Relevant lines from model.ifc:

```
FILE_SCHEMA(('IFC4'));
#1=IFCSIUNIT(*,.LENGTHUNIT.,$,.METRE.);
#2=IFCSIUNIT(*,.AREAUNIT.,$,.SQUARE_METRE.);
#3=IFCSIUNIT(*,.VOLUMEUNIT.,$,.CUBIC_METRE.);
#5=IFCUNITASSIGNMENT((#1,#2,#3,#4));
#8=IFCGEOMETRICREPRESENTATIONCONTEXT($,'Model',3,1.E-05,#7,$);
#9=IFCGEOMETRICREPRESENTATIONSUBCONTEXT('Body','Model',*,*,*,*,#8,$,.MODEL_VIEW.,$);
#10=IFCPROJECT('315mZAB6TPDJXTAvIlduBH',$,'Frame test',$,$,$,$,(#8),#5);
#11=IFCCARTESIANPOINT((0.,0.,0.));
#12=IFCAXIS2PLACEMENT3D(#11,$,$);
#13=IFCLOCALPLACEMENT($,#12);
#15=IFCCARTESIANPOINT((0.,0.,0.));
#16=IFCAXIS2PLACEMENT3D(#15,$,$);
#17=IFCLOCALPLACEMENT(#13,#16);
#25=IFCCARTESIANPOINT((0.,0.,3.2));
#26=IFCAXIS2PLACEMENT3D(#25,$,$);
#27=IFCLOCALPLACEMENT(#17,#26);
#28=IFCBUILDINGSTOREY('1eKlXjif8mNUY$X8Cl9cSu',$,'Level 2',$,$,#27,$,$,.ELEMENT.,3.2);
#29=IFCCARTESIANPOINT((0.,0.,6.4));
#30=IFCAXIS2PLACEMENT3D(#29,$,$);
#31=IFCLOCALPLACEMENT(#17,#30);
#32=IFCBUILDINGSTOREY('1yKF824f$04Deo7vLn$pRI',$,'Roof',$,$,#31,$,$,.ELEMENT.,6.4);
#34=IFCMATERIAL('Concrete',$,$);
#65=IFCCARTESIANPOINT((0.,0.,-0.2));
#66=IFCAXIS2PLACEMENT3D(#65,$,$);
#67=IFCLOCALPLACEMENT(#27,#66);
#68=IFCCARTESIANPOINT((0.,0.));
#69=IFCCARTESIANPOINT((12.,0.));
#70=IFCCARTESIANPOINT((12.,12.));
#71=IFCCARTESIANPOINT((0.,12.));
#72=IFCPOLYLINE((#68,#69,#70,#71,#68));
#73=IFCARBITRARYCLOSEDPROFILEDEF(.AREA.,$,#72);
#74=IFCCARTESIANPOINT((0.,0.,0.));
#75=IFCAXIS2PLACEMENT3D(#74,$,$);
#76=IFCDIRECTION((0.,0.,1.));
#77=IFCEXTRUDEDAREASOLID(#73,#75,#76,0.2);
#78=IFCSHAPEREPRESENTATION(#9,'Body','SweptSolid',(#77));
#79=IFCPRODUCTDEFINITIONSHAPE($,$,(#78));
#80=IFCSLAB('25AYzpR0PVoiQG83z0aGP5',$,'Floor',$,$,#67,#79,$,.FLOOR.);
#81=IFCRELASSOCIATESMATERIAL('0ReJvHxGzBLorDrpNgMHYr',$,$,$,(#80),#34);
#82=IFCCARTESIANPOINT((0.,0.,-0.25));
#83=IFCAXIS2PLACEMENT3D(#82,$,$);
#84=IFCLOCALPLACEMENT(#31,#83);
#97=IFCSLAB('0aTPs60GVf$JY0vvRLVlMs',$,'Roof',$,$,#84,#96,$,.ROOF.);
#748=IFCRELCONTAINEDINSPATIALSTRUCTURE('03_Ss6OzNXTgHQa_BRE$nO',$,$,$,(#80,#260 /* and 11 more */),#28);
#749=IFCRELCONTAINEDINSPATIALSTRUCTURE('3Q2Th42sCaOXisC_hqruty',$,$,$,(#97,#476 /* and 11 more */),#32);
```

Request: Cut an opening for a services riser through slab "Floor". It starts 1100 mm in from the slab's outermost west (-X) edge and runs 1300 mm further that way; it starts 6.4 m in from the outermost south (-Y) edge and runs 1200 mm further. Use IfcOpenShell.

```python
import numpy as np
import ifcopenshell
import ifcopenshell.api.feature
import ifcopenshell.api.geometry
import ifcopenshell.api.root
import ifcopenshell.geom
import ifcopenshell.util.placement
import ifcopenshell.util.representation
import ifcopenshell.util.shape
import ifcopenshell.util.unit

model = ifcopenshell.open("model.ifc")
unit_scale = ifcopenshell.util.unit.calculate_unit_scale(model)
settings = ifcopenshell.geom.settings()


def volume(element):
    """Net volume in cubic metres, openings subtracted."""
    shape = ifcopenshell.geom.create_shape(settings, element)
    return ifcopenshell.util.shape.get_volume(shape.geometry)


slab = model.by_guid("25AYzpR0PVoiQG83z0aGP5")
before = volume(slab)

# Extent in the slab's own axes, in metres. The edges named are its -X and -Y sides.
slab_shape = ifcopenshell.geom.create_shape(settings, slab)
vertices = ifcopenshell.util.shape.get_vertices(slab_shape.geometry)
x_min, y_min, bottom = vertices.min(axis=0)
top = vertices[:, 2].max()

opening = ifcopenshell.api.root.create_entity(model, ifc_class="IfcOpeningElement", name="Services riser opening", predefined_type="OPENING")
context = ifcopenshell.util.representation.get_context(model, "Model", "Body", "MODEL_VIEW")
width, depth = 1.3, 1.2
outline = [(0.0, 0.0), (width, 0.0), (width, depth), (0.0, depth), (0.0, 0.0)]
# Overshoot both faces by 50 mm so the cut is clean.
shape = ifcopenshell.api.geometry.add_slab_representation(
    model, context=context, depth=top - bottom + 0.1, polyline=outline
)
ifcopenshell.api.geometry.assign_representation(model, product=opening, representation=shape)

matrix = ifcopenshell.util.placement.get_local_placement(slab.ObjectPlacement)
matrix[:, 3] = matrix @ np.append(np.array([x_min + 1.1, y_min + 6.4, bottom - 0.05]) / unit_scale, 1.0)
ifcopenshell.api.geometry.edit_object_placement(model, product=opening, matrix=matrix, is_si=False)
ifcopenshell.api.feature.add_feature(model, feature=opening, element=slab)

after = volume(slab)

print(f"slab volume {before:.3f} -> {after:.3f} m3")

model.write("model_updated.ifc")
```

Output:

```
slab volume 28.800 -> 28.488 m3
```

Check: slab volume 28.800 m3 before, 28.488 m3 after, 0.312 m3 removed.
